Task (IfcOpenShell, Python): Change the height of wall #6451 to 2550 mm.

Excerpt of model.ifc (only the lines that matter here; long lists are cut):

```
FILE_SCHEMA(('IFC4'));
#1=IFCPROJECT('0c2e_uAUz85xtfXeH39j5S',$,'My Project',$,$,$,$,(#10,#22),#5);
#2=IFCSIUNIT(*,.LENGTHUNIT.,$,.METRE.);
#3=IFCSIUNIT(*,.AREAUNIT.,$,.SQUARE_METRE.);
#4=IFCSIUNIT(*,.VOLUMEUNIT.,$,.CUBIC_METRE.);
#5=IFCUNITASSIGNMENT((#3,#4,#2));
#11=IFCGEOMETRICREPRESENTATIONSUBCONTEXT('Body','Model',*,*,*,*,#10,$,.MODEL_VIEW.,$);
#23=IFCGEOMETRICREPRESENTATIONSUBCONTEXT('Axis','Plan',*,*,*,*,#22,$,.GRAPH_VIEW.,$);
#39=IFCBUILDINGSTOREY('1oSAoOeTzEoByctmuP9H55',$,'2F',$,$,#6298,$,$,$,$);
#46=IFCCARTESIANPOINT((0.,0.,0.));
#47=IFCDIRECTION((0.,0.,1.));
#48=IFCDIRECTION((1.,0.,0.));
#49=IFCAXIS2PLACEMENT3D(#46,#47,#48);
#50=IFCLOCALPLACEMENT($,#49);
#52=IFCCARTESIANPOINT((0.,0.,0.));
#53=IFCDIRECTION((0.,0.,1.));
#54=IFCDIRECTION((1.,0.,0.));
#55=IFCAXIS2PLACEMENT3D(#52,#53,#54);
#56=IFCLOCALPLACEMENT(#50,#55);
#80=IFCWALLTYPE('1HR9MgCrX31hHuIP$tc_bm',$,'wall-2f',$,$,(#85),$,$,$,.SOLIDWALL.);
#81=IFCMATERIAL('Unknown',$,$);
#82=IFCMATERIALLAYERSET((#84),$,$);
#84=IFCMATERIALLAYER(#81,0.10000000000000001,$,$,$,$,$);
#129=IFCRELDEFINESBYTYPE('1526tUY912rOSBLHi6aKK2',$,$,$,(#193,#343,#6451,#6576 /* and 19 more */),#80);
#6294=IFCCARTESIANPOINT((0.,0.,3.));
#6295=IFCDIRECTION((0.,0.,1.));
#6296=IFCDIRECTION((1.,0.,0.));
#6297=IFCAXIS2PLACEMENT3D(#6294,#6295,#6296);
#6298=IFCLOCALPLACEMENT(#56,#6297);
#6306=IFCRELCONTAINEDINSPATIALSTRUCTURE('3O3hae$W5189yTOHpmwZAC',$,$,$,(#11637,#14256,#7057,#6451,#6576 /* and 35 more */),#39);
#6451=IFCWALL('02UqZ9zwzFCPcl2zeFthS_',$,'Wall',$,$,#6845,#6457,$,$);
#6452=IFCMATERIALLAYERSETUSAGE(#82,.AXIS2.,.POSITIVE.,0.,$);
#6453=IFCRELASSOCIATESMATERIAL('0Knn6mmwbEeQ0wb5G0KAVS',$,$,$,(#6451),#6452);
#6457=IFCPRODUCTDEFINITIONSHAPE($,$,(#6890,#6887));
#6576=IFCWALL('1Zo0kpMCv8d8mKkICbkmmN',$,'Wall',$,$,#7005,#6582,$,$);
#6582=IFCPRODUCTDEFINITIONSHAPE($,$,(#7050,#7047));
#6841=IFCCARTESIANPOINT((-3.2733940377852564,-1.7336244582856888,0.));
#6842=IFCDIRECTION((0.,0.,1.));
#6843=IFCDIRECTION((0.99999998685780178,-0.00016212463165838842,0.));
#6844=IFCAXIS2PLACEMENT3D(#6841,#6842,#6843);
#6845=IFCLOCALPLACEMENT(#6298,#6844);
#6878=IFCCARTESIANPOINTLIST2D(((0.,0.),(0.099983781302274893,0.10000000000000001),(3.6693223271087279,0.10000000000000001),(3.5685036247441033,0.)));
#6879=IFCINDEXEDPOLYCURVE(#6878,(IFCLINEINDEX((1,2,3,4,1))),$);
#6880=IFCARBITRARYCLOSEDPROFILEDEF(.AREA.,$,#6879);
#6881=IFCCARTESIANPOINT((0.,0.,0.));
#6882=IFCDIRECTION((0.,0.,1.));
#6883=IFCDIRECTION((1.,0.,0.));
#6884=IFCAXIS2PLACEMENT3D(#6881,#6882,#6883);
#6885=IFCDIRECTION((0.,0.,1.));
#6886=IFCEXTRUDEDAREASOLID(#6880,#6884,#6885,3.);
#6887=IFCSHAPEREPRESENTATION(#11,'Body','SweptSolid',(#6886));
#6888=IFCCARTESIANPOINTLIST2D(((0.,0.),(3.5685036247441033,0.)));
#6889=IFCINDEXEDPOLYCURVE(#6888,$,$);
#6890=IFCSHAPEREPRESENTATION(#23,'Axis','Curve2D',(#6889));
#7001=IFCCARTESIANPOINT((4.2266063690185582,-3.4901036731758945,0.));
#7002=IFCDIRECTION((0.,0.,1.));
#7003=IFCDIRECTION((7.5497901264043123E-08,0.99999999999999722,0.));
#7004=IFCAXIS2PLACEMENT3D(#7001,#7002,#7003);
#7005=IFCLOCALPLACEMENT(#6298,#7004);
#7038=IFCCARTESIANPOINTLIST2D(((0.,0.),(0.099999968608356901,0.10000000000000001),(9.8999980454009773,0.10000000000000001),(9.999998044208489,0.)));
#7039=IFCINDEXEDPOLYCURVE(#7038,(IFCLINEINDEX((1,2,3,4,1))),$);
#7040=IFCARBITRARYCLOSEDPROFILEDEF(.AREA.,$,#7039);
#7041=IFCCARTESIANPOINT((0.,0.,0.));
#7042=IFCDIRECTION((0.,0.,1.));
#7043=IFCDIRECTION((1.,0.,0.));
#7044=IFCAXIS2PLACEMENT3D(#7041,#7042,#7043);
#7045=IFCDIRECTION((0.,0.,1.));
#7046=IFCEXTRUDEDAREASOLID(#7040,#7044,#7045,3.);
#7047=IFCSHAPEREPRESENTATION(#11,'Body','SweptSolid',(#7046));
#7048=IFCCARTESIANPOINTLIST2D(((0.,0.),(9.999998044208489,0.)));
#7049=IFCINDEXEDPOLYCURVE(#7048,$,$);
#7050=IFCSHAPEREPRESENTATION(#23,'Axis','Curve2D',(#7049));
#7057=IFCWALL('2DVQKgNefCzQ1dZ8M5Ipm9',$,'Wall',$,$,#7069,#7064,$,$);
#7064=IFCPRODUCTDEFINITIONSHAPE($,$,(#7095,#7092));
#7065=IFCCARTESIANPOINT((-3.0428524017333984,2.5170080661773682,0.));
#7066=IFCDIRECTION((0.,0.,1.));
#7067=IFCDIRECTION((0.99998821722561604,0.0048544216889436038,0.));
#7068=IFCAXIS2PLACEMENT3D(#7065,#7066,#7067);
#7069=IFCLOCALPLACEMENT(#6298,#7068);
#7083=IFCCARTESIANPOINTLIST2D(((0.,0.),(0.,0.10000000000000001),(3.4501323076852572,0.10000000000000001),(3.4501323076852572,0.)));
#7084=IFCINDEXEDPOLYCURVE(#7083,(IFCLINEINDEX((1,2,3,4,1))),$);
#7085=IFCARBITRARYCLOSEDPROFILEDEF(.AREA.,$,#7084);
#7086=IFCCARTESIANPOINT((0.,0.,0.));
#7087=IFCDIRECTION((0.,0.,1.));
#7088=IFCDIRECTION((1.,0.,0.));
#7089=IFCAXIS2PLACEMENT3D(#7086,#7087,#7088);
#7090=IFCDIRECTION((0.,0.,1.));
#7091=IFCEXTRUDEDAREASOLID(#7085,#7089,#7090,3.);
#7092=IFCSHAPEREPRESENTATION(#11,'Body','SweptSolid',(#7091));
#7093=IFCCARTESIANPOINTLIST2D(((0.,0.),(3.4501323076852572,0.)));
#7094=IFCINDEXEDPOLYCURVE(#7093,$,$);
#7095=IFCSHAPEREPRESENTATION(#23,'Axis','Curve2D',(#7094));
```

```python
import ifcopenshell
import ifcopenshell.geom
import ifcopenshell.util.representation
import ifcopenshell.util.shape

model = ifcopenshell.open("model.ifc")
settings = ifcopenshell.geom.settings()


def volume(element):
    """Net volume in cubic metres, openings subtracted."""
    shape = ifcopenshell.geom.create_shape(settings, element)
    return ifcopenshell.util.shape.get_volume(shape.geometry)


wall = model.by_guid("02UqZ9zwzFCPcl2zeFthS_")
before = volume(wall)

body = ifcopenshell.util.representation.get_representation(wall, "Model", "Body")
solid = body.Items[0]
old_height = solid.Depth
solid.Depth = 2.55
after = volume(wall)

print(f"height {old_height:g} -> {solid.Depth:g}, volume {before:.3f} -> {after:.3f} m3")

model.write("model_rev.ifc")
```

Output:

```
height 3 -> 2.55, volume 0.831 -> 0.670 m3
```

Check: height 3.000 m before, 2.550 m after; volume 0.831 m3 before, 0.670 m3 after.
